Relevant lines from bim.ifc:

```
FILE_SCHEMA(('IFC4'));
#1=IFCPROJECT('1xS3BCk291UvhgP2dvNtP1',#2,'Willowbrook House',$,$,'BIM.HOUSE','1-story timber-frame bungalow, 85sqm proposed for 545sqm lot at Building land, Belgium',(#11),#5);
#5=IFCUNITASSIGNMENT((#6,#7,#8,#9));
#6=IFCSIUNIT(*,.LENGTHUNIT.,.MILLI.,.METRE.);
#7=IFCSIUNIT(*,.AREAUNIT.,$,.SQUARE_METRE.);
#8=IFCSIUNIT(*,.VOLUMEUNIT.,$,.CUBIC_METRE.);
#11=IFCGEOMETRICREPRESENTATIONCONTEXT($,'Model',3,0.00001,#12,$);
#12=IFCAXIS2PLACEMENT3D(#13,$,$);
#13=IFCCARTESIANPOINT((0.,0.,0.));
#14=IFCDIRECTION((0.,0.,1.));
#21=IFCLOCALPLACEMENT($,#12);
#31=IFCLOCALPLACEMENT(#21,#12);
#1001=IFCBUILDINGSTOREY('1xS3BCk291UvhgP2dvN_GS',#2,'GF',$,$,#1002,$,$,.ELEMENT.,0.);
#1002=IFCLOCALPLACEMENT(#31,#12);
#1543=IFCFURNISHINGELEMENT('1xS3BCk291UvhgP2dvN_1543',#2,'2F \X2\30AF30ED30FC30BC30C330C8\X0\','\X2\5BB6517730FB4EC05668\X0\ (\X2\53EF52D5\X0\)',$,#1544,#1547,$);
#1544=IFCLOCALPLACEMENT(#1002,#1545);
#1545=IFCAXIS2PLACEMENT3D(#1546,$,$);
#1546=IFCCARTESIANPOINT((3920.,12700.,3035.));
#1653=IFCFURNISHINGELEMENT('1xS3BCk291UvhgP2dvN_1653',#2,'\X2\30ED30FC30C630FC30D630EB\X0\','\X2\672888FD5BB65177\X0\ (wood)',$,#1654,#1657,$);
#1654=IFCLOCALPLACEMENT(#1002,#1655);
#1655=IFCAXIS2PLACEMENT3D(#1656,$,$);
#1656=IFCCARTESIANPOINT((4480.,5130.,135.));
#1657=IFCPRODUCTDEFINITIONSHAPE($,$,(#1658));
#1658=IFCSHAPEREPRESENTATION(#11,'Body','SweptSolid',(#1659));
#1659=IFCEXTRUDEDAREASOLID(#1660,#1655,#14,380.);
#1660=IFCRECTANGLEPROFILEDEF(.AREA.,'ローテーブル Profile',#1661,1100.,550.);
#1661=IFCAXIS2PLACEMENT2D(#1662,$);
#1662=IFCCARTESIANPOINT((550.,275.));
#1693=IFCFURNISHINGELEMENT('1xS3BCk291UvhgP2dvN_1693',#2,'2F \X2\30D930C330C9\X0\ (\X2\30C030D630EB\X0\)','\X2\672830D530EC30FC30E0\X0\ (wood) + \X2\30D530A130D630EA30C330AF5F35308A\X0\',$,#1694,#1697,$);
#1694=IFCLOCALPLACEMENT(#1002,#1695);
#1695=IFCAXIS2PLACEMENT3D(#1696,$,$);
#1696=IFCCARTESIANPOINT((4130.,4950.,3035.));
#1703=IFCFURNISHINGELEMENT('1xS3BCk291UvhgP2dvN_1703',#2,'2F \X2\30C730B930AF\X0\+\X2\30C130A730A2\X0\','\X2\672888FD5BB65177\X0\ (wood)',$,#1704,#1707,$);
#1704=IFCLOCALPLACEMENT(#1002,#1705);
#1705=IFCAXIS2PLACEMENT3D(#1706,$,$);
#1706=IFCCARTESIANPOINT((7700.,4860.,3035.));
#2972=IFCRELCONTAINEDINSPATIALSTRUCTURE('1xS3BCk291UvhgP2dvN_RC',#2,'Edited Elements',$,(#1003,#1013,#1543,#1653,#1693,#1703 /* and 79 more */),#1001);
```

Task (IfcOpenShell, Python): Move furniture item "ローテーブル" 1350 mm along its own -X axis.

```python
import ifcopenshell
import ifcopenshell.api.geometry
import ifcopenshell.util.placement

model = ifcopenshell.open("bim.ifc")

item = model.by_id(1653)
matrix = ifcopenshell.util.placement.get_local_placement(item.ObjectPlacement)
matrix[:3, 3] -= matrix[:3, 0] * 1350.0
ifcopenshell.api.geometry.edit_object_placement(model, product=item, matrix=matrix, is_si=False)

print(ifcopenshell.util.placement.get_local_placement(item.ObjectPlacement).round(3) + 0.0)

model.write("bim_v2.ifc")
```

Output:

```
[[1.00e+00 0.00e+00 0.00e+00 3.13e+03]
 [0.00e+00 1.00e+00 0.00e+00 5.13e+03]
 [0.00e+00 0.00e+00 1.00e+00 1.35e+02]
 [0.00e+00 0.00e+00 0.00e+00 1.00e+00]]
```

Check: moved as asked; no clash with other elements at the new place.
